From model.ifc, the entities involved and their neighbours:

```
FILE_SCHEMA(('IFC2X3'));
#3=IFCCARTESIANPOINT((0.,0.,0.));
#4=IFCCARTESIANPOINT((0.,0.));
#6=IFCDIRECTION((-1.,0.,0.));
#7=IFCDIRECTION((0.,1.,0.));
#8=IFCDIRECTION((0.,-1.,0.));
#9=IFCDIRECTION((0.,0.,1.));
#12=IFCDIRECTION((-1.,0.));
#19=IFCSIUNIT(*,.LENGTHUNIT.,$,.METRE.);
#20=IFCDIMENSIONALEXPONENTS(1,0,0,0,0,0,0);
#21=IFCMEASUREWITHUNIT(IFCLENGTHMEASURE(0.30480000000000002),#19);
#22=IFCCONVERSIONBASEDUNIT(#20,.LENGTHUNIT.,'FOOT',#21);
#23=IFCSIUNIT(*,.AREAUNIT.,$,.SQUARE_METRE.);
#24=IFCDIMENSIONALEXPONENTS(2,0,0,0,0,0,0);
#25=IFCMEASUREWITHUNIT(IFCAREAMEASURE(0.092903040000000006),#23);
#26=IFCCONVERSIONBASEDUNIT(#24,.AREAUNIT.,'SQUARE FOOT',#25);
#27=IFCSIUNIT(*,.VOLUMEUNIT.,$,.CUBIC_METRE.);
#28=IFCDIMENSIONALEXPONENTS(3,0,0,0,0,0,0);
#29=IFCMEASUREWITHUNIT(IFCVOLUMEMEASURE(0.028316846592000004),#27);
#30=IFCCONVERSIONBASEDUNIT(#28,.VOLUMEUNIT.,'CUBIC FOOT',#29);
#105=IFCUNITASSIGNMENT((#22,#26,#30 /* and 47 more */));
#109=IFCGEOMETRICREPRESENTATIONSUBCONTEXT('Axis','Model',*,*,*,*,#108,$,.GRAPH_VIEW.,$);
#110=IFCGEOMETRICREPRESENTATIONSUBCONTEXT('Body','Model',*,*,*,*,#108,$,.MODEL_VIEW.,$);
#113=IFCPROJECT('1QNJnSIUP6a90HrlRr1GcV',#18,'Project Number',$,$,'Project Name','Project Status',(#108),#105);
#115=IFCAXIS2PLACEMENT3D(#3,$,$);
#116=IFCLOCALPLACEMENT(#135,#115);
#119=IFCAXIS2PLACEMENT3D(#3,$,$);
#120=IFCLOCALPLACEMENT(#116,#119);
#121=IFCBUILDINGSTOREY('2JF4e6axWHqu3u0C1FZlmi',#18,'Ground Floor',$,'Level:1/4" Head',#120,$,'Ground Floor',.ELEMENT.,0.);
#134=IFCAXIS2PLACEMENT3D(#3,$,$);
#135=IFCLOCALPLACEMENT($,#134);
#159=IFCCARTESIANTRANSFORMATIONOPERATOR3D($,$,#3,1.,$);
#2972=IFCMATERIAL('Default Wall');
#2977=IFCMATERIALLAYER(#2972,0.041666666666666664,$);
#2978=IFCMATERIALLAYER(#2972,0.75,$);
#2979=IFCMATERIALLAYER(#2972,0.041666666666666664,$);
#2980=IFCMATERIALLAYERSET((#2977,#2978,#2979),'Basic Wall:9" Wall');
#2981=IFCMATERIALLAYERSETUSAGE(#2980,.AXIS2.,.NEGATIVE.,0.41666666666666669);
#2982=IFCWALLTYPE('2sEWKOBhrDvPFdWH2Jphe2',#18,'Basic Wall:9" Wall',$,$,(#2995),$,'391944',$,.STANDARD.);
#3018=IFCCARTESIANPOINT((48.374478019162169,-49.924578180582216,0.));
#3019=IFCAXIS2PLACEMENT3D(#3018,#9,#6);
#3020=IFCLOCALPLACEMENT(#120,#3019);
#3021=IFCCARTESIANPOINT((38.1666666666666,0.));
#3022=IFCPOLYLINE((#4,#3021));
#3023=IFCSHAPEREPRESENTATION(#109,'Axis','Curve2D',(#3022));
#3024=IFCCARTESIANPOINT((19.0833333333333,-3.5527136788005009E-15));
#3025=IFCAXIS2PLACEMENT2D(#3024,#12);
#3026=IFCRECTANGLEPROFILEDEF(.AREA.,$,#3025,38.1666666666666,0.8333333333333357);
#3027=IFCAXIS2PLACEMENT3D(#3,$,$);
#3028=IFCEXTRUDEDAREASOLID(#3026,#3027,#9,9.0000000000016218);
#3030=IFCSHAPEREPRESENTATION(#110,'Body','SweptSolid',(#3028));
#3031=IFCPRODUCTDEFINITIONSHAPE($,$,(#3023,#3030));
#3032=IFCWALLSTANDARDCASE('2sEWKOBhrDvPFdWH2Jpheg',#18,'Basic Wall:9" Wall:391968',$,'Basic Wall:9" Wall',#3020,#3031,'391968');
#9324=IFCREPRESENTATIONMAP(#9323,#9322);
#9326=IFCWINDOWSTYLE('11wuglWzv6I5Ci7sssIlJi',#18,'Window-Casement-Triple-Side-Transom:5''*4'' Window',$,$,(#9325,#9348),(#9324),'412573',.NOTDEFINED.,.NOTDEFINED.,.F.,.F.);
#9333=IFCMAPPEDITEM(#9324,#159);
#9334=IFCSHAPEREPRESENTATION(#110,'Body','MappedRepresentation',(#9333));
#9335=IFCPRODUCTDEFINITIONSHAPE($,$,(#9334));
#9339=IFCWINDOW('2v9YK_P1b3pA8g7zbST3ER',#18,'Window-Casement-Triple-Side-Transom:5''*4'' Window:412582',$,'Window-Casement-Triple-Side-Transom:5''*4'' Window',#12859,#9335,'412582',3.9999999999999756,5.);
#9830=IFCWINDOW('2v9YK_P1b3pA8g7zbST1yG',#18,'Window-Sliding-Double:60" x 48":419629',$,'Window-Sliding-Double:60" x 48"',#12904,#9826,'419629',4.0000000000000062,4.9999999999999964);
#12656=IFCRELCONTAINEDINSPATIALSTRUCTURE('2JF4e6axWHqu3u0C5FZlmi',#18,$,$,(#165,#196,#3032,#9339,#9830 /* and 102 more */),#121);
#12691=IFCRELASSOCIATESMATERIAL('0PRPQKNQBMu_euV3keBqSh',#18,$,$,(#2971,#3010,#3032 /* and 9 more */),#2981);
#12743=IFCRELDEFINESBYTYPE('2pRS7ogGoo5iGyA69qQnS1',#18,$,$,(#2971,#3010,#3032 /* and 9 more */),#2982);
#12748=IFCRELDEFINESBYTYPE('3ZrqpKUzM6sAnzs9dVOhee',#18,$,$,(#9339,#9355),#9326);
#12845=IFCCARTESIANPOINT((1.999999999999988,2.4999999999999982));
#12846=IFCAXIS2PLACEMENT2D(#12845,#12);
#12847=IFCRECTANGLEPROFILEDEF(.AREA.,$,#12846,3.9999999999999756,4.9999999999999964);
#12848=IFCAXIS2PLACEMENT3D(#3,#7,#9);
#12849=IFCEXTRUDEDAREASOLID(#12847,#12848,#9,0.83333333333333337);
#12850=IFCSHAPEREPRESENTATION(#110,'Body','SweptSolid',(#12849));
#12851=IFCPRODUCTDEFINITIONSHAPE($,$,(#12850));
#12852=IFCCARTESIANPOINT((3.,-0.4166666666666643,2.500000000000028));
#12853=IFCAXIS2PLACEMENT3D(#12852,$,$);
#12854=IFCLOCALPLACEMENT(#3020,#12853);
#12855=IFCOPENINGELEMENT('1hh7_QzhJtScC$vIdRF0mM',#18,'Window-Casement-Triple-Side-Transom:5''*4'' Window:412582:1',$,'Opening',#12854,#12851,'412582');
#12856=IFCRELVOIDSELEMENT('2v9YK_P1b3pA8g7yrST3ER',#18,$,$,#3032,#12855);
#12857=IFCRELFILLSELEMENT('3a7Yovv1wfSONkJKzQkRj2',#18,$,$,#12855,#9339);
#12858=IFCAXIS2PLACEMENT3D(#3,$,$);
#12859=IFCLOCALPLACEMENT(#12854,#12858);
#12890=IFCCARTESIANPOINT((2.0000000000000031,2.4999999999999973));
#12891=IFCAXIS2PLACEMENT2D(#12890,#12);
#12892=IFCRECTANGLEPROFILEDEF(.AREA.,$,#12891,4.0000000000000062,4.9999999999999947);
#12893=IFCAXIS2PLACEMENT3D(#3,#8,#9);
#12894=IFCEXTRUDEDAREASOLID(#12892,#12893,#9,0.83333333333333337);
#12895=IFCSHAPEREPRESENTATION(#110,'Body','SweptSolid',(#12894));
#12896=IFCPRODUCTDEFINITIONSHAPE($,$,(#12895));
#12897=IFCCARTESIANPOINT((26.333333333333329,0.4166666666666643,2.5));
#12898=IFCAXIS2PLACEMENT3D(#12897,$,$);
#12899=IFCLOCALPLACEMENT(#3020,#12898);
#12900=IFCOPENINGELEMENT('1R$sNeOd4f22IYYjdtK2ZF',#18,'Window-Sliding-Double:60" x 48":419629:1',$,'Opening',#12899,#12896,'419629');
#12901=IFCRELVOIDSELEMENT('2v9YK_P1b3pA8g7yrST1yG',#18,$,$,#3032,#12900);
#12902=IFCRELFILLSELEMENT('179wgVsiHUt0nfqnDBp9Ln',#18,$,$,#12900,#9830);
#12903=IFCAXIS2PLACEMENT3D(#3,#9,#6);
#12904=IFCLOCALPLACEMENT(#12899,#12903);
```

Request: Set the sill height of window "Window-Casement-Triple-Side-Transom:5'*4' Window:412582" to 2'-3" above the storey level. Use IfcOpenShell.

```python
import numpy as np
import ifcopenshell
import ifcopenshell.api.geometry
import ifcopenshell.geom
import ifcopenshell.util.element
import ifcopenshell.util.placement
import ifcopenshell.util.shape
import ifcopenshell.util.unit

model = ifcopenshell.open("model.ifc")
unit_scale = ifcopenshell.util.unit.calculate_unit_scale(model)

window = model.by_guid("2v9YK_P1b3pA8g7zbST3ER")
opening = window.FillsVoids[0].RelatingOpeningElement
storey = ifcopenshell.util.element.get_container(window, ifc_class="IfcBuildingStorey")
level = ifcopenshell.util.placement.get_local_placement(storey.ObjectPlacement)[2, 3]

# The opening's origin need not be at the sill, so measure its lowest point.
shape = ifcopenshell.geom.create_shape(ifcopenshell.geom.settings(), opening)
bottom = ifcopenshell.util.shape.get_shape_bottom_elevation(shape, shape.geometry) / unit_scale
dz = level + 27 * 0.0254 / unit_scale - bottom

shift = np.array([0.0, 0.0, dz])
# The window is placed relative to its opening, so it follows when the opening moves.
matrix = ifcopenshell.util.placement.get_local_placement(opening.ObjectPlacement)
matrix[:3, 3] += shift
ifcopenshell.api.geometry.edit_object_placement(
    model, product=opening, matrix=matrix, is_si=False, should_transform_children=True
)

print(f"moved by {dz * unit_scale:+.3f} m")

model.write("model_edited.ifc")
```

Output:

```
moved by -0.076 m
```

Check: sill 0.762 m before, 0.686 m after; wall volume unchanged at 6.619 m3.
